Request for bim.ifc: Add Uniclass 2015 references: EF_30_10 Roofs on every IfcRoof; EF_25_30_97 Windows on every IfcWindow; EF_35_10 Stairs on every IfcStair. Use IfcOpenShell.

First a look at what the model holds.

```python
import ifcopenshell

model = ifcopenshell.open("bim.ifc")
print(model.schema)
print("classifications:", [c.Name for c in model.by_type("IfcClassification")])
for ifc_class in ("IfcDoor", "IfcRoof", "IfcStair", "IfcWall", "IfcWindow"):
    print(ifc_class, len(model.by_type(ifc_class)))
```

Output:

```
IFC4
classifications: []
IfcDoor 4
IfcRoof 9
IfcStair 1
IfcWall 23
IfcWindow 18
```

```python
import ifcopenshell
import ifcopenshell.api.classification

model = ifcopenshell.open("bim.ifc")

system = ifcopenshell.api.classification.add_classification(model, classification="Uniclass 2015")

codes = {
    "IfcRoof": ("EF_30_10", "Roofs"),
    "IfcWindow": ("EF_25_30_97", "Windows"),
    "IfcStair": ("EF_35_10", "Stairs"),
}
for ifc_class, (code, name) in codes.items():
    products = model.by_type(ifc_class)
    ifcopenshell.api.classification.add_reference(
        model, products=products, classification=system, identification=code, name=name
    )
    print(code, len(products))

model.write("bim_v2.ifc")
```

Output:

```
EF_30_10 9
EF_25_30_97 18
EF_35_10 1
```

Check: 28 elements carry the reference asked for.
